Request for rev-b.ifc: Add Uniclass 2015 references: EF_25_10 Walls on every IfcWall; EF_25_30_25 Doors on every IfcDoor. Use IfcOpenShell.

First a look at what the model holds.

```python
import ifcopenshell

model = ifcopenshell.open("rev-b.ifc")
print(model.schema)
print("classifications:", [c.Name for c in model.by_type("IfcClassification")])
for ifc_class in ("IfcDoor", "IfcRoof", "IfcStair", "IfcWall", "IfcWindow"):
    print(ifc_class, len(model.by_type(ifc_class)))
```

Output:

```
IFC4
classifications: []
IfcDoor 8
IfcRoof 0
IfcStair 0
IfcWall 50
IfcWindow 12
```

```python
import ifcopenshell
import ifcopenshell.api.classification

model = ifcopenshell.open("rev-b.ifc")

system = ifcopenshell.api.classification.add_classification(model, classification="Uniclass 2015")

codes = {
    "IfcWall": ("EF_25_10", "Walls"),
    "IfcDoor": ("EF_25_30_25", "Doors"),
}
for ifc_class, (code, name) in codes.items():
    products = model.by_type(ifc_class)
    ifcopenshell.api.classification.add_reference(
        model, products=products, classification=system, identification=code, name=name
    )
    print(code, len(products))

model.write("rev-b_edited.ifc")
```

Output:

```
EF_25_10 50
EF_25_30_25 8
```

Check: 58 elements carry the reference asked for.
